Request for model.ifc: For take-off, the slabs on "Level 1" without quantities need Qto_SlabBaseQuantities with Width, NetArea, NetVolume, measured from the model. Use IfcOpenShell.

First a look at what the model holds.

```python
import ifcopenshell
import ifcopenshell.util.element
import ifcopenshell.util.unit

model = ifcopenshell.open("model.ifc")
print(model.schema)
for unit_type in ("LENGTHUNIT", "AREAUNIT", "VOLUMEUNIT"):
    print(unit_type, ifcopenshell.util.unit.calculate_unit_scale(model, unit_type))
storey = next(s for s in model.by_type("IfcBuildingStorey") if s.Name == "Level 1")
slabs = [e for e in ifcopenshell.util.element.get_decomposition(storey) if e.is_a("IfcSlab")]
for e in sorted(slabs, key=lambda e: e.id()):
    print(e.id(), e.is_a(), e.Name, list(ifcopenshell.util.element.get_psets(e, qtos_only=True)), sep=" | ")
```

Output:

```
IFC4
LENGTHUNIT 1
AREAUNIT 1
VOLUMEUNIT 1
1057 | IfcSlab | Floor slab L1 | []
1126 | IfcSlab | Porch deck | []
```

```python
import ifcopenshell
import ifcopenshell.api.pset
import ifcopenshell.geom
import ifcopenshell.util.element
import ifcopenshell.util.shape
import ifcopenshell.util.unit

model = ifcopenshell.open("model.ifc")
unit_scale = ifcopenshell.util.unit.calculate_unit_scale(model)
area_scale = ifcopenshell.util.unit.calculate_unit_scale(model, "AREAUNIT")
volume_scale = ifcopenshell.util.unit.calculate_unit_scale(model, "VOLUMEUNIT")
settings = ifcopenshell.geom.settings()

storey = next(s for s in model.by_type("IfcBuildingStorey") if s.Name == "Level 1")
slabs = [e for e in ifcopenshell.util.element.get_decomposition(storey) if e.is_a("IfcSlab")]

for e in sorted(slabs, key=lambda e: e.id()):
    if ifcopenshell.util.element.get_psets(e, qtos_only=True, should_inherit=False):
        continue
    # Geometry comes back in metres, in the element's own axes.
    shape = ifcopenshell.geom.create_shape(settings, e)
    values = {
        "Width": ifcopenshell.util.shape.get_z(shape.geometry) / unit_scale,
        "NetArea": ifcopenshell.util.shape.get_footprint_area(shape.geometry) / area_scale,
        "NetVolume": ifcopenshell.util.shape.get_volume(shape.geometry) / volume_scale,
    }
    qto = ifcopenshell.api.pset.add_qto(model, product=e, name="Qto_SlabBaseQuantities")
    ifcopenshell.api.pset.edit_qto(model, qto=qto, properties=values)
    print(e.id(), {k: round(v, 3) for k, v in values.items()})

model.write("model_updated.ifc")
```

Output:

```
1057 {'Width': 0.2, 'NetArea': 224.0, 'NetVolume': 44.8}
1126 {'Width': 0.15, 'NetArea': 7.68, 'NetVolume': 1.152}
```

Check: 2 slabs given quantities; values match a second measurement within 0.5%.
